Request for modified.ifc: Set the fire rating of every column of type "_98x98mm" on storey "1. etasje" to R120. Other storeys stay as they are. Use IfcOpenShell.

First a look at what the model holds.

```python
import ifcopenshell
import ifcopenshell.util.element

model = ifcopenshell.open("modified.ifc")
print(model.schema)
storey = next(s for s in model.by_type("IfcBuildingStorey") if s.Name == "1. etasje")
columns = [e for e in ifcopenshell.util.element.get_decomposition(storey) if e.is_a("IfcColumn")]
seen = {}
for e in columns:
    element_type = ifcopenshell.util.element.get_type(e)
    key = (element_type.Name if element_type != e and element_type else None, ifcopenshell.util.element.get_pset(e, "Pset_ColumnCommon", "FireRating"))
    seen[key] = seen.get(key, 0) + 1
for (name, value), count in sorted(seen.items(), key=str):
    print(count, "x", name, "|", value)
```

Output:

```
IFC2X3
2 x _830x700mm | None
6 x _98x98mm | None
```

```python
import ifcopenshell
import ifcopenshell.api.pset
import ifcopenshell.util.element

model = ifcopenshell.open("modified.ifc")

storey = next(s for s in model.by_type("IfcBuildingStorey") if s.Name == "1. etasje")
columns = [e for e in ifcopenshell.util.element.get_decomposition(storey) if e.is_a("IfcColumn")]

count = 0
for e in columns:
    element_type = ifcopenshell.util.element.get_type(e)
    if element_type in (None, e) or element_type.Name != "_98x98mm":
        continue
    # add_pset returns the element's existing set when there is one.
    pset = ifcopenshell.api.pset.add_pset(model, product=e, name="Pset_ColumnCommon")
    ifcopenshell.api.pset.edit_pset(model, pset=pset, properties={"FireRating": "R120"})
    count += 1

print(count, "columns updated")

model.write("modified_v2.ifc")
```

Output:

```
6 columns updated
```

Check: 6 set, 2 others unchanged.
